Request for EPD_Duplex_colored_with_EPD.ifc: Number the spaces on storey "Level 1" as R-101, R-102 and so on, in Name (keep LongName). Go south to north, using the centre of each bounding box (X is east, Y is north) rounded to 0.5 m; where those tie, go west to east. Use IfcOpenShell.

First a look at what the model holds.

```python
import ifcopenshell
import ifcopenshell.util.element
import ifcopenshell.util.placement

model = ifcopenshell.open("EPD_Duplex_colored_with_EPD.ifc")
print(model.schema)
storey = next(s for s in model.by_type("IfcBuildingStorey") if s.Name == "Level 1")
spaces = [e for e in ifcopenshell.util.element.get_decomposition(storey) if e.is_a("IfcSpace")]
for e in sorted(spaces, key=lambda e: e.id()):
    origin = ifcopenshell.util.placement.get_local_placement(e.ObjectPlacement)[:3, 3]
    print(e.id(), e.Name, e.LongName, origin.round(2) + 0.0, sep=" | ")
```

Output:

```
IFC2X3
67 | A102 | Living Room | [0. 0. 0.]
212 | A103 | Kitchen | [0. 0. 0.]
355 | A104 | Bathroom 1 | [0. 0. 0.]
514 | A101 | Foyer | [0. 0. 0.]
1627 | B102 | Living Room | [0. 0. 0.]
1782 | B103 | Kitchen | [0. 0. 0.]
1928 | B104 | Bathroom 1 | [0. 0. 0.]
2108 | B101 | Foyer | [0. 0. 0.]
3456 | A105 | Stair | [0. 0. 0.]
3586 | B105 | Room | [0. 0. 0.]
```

```python
import ifcopenshell
import ifcopenshell.geom
import ifcopenshell.util.element
import ifcopenshell.util.shape

model = ifcopenshell.open("EPD_Duplex_colored_with_EPD.ifc")
settings = ifcopenshell.geom.settings()
settings.set("use-world-coords", True)


def centre(element):
    shape = ifcopenshell.geom.create_shape(settings, element)
    return ifcopenshell.util.shape.get_bbox_centroid(shape.geometry)


storey = next(s for s in model.by_type("IfcBuildingStorey") if s.Name == "Level 1")
spaces = [e for e in ifcopenshell.util.element.get_decomposition(storey) if e.is_a("IfcSpace")]

# Insertion points can sit at a corner or the storey origin, so sort by the geometry (in metres).
centres = {e: centre(e) for e in spaces}
spaces.sort(key=lambda e: (round(centres[e][1] / 0.5), centres[e][0]))

for i, e in enumerate(spaces, start=1):
    number = f"R-1{i:02d}"
    e.Name = number
    print(e.id(), number)

model.write("EPD_Duplex_colored_with_EPD_updated.ifc")
```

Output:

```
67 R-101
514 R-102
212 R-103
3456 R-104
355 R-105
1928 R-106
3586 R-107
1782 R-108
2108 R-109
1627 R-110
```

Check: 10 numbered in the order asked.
